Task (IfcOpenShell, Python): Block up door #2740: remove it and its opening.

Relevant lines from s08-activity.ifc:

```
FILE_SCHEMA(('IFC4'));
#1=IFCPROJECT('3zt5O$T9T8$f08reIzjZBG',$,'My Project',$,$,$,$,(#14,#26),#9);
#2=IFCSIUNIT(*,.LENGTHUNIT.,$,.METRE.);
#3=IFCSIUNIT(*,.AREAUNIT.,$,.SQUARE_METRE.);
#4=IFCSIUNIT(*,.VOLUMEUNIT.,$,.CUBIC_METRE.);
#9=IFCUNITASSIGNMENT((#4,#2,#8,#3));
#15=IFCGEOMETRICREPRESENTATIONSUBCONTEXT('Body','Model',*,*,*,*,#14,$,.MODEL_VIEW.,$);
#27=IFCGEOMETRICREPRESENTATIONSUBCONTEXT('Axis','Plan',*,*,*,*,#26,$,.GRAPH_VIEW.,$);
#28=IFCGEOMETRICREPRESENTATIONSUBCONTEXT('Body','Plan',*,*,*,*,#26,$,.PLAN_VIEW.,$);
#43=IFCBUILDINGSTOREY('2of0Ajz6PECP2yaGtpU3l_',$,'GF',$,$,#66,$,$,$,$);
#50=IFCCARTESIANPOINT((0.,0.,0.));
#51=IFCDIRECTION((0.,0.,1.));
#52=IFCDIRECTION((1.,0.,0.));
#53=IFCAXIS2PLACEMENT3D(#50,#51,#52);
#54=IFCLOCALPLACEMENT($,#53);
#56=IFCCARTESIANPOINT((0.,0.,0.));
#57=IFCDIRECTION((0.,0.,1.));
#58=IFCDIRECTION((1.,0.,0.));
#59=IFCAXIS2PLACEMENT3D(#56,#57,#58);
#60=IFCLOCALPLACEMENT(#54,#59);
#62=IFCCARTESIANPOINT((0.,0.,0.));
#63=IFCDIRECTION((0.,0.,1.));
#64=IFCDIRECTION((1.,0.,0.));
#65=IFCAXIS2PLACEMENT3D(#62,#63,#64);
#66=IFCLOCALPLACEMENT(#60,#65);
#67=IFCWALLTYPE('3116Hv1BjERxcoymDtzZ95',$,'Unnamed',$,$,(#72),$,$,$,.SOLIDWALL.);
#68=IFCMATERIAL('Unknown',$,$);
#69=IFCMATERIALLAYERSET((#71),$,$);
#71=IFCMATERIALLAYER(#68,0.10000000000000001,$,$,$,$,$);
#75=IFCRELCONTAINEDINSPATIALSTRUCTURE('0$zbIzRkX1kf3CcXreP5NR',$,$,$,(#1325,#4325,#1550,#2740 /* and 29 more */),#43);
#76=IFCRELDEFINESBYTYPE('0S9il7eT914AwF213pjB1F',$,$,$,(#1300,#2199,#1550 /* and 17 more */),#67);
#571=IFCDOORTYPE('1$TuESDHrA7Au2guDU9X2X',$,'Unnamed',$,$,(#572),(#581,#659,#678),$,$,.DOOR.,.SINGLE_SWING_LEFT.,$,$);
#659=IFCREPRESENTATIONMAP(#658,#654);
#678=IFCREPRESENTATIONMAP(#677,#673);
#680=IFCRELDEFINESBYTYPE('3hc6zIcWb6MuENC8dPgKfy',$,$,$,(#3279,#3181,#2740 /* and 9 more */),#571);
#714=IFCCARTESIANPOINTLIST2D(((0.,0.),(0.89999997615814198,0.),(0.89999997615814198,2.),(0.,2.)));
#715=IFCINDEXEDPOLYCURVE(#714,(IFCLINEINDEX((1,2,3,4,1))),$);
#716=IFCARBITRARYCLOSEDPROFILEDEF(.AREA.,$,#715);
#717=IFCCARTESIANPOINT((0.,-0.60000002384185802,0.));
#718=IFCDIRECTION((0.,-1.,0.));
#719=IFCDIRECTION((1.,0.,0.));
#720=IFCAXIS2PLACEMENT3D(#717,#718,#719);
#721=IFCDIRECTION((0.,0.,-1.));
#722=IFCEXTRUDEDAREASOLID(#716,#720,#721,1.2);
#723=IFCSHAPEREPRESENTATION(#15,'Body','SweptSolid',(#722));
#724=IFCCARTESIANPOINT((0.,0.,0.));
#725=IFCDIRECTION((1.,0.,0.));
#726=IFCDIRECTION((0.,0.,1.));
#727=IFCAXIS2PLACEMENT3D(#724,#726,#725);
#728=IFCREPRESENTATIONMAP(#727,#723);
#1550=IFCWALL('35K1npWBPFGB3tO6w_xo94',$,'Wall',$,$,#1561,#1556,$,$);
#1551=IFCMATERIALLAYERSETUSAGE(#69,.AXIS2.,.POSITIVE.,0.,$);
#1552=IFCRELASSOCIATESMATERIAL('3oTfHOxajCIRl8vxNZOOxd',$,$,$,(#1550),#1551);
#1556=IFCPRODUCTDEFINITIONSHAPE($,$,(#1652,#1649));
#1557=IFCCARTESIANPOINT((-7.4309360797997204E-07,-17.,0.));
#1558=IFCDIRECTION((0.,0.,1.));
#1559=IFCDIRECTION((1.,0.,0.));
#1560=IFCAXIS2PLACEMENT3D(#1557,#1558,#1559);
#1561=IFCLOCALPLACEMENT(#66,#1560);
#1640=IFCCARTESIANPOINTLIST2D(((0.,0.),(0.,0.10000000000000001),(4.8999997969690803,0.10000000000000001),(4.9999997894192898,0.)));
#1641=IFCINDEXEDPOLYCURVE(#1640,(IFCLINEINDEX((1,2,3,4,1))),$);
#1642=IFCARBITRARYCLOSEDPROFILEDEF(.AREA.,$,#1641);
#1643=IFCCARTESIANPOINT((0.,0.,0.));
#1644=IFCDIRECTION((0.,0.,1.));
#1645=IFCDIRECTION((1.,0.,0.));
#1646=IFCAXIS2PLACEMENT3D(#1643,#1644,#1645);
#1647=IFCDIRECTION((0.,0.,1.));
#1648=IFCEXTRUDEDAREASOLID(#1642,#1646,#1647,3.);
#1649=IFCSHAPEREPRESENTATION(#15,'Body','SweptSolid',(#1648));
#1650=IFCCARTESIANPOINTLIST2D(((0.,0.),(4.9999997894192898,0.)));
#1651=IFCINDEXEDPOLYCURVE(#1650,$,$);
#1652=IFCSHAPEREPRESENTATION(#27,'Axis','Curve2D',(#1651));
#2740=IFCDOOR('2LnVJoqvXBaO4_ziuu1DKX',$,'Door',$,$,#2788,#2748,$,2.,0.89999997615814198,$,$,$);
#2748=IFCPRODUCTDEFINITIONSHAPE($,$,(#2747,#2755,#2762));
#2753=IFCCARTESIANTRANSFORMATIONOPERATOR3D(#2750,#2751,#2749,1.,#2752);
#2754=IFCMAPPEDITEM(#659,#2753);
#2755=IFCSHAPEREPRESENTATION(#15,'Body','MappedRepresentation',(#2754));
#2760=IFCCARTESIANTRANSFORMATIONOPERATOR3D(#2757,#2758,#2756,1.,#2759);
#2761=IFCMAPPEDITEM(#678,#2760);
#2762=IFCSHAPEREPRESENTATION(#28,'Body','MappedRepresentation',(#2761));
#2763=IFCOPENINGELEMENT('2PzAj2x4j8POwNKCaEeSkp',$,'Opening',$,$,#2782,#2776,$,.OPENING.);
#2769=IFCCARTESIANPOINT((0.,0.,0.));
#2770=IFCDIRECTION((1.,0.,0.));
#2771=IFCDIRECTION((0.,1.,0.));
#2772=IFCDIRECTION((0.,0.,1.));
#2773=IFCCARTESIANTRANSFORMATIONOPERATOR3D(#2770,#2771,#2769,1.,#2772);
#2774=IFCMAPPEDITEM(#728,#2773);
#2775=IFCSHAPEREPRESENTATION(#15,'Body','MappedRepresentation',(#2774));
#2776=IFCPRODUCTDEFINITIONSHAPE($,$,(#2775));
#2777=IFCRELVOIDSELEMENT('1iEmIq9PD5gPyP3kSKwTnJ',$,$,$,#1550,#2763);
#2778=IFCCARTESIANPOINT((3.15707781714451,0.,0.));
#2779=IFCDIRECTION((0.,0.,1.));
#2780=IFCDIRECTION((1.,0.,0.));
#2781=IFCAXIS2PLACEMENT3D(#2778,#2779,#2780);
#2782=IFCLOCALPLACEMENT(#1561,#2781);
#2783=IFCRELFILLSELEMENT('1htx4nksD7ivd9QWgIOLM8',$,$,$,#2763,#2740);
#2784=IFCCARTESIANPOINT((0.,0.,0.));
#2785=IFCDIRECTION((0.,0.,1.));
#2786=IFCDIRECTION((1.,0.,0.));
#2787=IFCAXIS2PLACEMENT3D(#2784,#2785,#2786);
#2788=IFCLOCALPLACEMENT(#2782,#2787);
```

```python
import ifcopenshell
import ifcopenshell.api.feature
import ifcopenshell.api.root
import ifcopenshell.geom
import ifcopenshell.util.shape

model = ifcopenshell.open("s08-activity.ifc")
settings = ifcopenshell.geom.settings()


def volume(element):
    """Net volume in cubic metres, openings subtracted."""
    shape = ifcopenshell.geom.create_shape(settings, element)
    return ifcopenshell.util.shape.get_volume(shape.geometry)


door = model.by_id(2740)
opening = door.FillsVoids[0].RelatingOpeningElement
wall = opening.VoidsElements[0].RelatingBuildingElement
before = volume(wall)

ifcopenshell.api.root.remove_product(model, product=door)
ifcopenshell.api.feature.remove_feature(model, feature=opening)

after = volume(wall)

print(f"wall volume {before:.3f} -> {after:.3f} m3")

model.write("s08-activity_updated.ifc")
```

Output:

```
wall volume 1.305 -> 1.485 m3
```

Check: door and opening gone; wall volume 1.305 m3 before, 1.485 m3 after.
